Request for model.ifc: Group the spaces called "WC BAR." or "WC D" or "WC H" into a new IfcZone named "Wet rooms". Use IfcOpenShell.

First a look at what the model holds.

```python
import ifcopenshell

model = ifcopenshell.open("model.ifc")
print(model.schema)
seen = {}
for space in model.by_type("IfcSpace"):
    seen[space.LongName] = seen.get(space.LongName, 0) + 1
for name, count in sorted(seen.items(), key=str):
    print(count, "x", name)
print("zones:", [z.Name for z in model.by_type("IfcZone")][:20])
```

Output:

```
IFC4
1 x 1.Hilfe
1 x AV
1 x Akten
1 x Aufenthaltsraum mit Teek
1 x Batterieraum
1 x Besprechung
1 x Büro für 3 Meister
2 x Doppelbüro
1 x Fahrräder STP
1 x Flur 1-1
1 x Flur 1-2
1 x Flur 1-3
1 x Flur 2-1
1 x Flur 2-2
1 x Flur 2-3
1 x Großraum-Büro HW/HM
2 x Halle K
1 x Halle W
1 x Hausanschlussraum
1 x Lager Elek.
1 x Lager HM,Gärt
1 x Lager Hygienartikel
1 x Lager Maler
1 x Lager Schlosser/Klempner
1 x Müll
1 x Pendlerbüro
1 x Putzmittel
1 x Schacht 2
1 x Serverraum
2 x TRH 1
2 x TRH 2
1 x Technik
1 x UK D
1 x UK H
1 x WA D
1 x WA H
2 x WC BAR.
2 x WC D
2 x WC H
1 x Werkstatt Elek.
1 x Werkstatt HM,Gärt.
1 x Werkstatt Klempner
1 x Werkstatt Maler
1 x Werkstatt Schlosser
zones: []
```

```python
import ifcopenshell
import ifcopenshell.api.group
import ifcopenshell.api.root

model = ifcopenshell.open("model.ifc")

names = {"WC BAR.", "WC D", "WC H"}
spaces = [s for s in model.by_type("IfcSpace") if s.LongName in names]

zone = ifcopenshell.api.root.create_entity(model, ifc_class="IfcZone", name="Wet rooms")
ifcopenshell.api.group.assign_group(model, products=spaces, group=zone)
print(len(spaces), "spaces in", zone.Name)

model.write("model-out.ifc")
```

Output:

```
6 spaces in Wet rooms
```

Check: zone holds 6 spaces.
